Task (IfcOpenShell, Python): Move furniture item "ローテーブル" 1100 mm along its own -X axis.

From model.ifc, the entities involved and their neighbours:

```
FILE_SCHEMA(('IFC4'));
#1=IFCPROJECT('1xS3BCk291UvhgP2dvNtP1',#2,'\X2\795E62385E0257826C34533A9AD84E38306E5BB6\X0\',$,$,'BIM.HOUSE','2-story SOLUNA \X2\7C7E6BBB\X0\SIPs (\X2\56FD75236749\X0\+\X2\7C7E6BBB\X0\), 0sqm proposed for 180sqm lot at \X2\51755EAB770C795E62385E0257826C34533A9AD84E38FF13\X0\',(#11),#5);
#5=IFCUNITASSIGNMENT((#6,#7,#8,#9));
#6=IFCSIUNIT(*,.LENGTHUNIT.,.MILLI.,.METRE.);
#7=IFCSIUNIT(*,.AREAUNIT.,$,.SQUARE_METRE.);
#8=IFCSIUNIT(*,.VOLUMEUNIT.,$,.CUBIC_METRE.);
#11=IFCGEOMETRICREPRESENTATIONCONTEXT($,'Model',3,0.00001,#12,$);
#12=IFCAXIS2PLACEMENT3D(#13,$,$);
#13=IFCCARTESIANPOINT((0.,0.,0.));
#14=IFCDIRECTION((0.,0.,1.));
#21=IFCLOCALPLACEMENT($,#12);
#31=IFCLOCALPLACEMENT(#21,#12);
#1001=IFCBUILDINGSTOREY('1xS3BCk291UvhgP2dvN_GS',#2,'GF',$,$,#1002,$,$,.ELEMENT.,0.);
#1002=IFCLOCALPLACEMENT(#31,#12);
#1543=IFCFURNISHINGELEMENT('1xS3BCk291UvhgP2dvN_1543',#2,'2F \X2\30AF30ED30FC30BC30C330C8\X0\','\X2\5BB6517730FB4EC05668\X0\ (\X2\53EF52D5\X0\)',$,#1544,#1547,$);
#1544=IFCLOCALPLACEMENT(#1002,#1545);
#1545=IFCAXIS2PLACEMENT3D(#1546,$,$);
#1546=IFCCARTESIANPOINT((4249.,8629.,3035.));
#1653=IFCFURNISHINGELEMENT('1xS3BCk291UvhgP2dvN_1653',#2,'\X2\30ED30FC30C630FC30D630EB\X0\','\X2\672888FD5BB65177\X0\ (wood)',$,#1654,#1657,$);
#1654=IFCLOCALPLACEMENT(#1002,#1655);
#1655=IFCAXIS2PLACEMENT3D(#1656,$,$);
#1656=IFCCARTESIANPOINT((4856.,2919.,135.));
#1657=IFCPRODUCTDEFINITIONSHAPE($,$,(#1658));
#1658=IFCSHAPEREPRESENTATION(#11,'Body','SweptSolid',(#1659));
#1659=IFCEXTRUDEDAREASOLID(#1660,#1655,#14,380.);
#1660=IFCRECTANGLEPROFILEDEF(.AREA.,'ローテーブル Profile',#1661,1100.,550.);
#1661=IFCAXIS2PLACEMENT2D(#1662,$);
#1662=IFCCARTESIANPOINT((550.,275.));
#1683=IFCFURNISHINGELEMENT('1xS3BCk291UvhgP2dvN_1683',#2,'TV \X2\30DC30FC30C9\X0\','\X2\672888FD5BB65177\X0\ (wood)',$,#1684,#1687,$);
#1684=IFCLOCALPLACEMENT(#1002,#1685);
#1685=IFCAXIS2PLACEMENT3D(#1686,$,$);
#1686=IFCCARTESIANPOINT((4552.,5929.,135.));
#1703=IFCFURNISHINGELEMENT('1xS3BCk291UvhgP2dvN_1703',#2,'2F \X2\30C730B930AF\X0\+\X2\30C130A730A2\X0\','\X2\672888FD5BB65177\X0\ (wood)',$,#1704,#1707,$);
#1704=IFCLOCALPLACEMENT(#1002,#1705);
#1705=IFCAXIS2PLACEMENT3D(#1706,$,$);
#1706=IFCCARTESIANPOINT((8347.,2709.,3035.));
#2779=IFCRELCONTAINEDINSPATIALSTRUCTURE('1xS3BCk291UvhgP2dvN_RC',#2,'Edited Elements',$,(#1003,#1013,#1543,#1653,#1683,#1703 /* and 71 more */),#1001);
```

```python
import ifcopenshell
import ifcopenshell.api.geometry
import ifcopenshell.util.placement

model = ifcopenshell.open("model.ifc")

item = model.by_guid("1xS3BCk291UvhgP2dvN_1653")
matrix = ifcopenshell.util.placement.get_local_placement(item.ObjectPlacement)
matrix[:3, 3] -= matrix[:3, 0] * 1100.0
ifcopenshell.api.geometry.edit_object_placement(model, product=item, matrix=matrix, is_si=False)

print(ifcopenshell.util.placement.get_local_placement(item.ObjectPlacement).round(3) + 0.0)

model.write("model-out.ifc")
```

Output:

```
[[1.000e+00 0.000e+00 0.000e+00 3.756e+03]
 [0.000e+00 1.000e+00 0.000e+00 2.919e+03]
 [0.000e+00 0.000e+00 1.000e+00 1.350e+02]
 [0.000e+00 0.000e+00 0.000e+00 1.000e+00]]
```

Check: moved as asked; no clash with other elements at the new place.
